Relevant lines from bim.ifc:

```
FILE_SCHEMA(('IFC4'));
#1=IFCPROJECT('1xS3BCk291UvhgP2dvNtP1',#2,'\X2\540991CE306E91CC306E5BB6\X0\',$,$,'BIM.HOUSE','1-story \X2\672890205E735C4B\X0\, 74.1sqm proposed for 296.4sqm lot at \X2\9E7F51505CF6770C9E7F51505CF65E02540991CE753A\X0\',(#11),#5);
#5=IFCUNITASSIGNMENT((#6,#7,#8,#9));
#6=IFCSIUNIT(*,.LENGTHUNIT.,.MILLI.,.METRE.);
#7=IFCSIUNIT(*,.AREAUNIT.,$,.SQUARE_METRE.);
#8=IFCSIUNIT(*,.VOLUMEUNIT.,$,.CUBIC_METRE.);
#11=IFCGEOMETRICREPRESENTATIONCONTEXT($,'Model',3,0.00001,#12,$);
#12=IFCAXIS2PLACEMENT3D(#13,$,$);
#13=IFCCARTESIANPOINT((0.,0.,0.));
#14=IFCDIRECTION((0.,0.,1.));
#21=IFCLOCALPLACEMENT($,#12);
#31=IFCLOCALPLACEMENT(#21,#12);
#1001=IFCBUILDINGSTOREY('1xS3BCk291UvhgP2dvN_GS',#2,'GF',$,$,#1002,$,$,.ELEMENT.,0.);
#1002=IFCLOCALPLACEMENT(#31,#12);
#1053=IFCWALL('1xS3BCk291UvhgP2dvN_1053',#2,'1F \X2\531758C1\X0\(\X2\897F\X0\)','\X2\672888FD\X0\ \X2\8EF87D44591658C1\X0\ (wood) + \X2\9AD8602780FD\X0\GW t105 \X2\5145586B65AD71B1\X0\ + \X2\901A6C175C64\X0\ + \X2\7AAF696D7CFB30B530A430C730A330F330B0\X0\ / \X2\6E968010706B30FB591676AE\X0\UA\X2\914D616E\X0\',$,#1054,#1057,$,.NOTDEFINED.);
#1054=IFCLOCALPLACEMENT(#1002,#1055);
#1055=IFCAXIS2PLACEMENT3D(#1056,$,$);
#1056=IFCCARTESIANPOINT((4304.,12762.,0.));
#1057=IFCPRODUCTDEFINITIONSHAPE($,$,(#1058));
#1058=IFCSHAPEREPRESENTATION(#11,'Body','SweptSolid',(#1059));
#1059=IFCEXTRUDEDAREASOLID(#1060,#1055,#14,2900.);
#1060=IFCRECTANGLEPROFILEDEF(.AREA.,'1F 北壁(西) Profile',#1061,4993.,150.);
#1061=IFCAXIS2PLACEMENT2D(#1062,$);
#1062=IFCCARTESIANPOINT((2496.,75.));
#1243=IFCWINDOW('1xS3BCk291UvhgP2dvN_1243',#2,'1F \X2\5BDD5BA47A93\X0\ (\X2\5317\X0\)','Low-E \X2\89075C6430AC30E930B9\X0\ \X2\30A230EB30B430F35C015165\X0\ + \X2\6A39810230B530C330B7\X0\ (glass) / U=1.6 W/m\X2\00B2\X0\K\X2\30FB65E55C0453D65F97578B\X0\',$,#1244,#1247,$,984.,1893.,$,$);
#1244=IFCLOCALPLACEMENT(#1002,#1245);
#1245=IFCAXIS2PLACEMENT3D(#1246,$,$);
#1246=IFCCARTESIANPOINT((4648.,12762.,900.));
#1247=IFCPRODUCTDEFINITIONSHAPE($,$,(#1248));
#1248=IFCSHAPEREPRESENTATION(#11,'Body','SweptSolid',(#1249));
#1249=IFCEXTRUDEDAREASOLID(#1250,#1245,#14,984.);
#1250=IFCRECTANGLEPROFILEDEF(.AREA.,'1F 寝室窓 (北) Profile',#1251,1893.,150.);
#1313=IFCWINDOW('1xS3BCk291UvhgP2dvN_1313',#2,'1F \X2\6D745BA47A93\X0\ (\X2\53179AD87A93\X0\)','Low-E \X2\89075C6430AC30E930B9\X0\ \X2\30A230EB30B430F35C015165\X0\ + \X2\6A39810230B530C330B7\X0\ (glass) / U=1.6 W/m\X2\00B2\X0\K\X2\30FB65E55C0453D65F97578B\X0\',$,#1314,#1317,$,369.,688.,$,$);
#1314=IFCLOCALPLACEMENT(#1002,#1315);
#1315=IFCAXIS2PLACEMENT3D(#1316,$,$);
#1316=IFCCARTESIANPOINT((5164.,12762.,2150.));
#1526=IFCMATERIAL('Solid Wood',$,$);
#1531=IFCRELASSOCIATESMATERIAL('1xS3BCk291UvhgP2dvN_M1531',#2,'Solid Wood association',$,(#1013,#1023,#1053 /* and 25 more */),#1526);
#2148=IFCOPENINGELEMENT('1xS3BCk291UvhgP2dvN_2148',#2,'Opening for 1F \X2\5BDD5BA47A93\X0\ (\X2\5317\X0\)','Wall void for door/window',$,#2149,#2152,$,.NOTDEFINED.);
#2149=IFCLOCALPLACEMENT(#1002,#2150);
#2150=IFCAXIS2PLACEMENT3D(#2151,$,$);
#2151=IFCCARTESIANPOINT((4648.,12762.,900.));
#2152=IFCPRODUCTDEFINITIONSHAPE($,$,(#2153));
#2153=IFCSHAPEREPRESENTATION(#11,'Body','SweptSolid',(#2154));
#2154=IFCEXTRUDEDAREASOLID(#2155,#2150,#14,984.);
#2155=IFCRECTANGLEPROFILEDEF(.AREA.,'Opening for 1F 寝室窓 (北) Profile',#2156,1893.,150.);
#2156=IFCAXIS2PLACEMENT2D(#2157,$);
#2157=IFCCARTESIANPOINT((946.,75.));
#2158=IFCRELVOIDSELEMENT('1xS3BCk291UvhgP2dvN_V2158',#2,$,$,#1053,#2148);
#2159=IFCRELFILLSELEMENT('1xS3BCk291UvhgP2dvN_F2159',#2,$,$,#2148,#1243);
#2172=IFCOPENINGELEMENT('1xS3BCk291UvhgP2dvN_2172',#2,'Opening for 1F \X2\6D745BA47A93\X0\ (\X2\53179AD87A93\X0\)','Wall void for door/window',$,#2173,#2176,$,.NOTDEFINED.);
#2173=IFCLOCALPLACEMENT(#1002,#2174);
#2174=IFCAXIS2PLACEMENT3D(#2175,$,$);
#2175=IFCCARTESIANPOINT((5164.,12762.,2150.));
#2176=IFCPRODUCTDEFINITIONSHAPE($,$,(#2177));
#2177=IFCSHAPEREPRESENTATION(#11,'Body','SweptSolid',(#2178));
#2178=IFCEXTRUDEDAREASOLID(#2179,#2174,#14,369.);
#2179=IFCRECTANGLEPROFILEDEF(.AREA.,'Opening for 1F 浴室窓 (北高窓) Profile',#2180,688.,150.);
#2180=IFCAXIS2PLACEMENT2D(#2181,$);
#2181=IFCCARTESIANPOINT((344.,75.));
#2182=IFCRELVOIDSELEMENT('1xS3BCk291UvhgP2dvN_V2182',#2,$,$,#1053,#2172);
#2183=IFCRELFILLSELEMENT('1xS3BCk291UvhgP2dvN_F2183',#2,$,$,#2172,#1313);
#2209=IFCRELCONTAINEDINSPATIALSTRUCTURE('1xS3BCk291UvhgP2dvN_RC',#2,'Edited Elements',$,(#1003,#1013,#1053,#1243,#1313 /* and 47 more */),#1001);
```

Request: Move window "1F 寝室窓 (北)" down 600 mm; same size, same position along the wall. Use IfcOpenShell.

```python
import numpy as np
import ifcopenshell
import ifcopenshell.api.geometry
import ifcopenshell.util.placement
import ifcopenshell.util.unit

model = ifcopenshell.open("bim.ifc")
unit_scale = ifcopenshell.util.unit.calculate_unit_scale(model)

window = model.by_guid("1xS3BCk291UvhgP2dvN_1243")
opening = window.FillsVoids[0].RelatingOpeningElement
dz = -0.6 / unit_scale

shift = np.array([0.0, 0.0, dz])
# The window is not placed relative to its opening, so move both.
for product in (opening, window):
    matrix = ifcopenshell.util.placement.get_local_placement(product.ObjectPlacement)
    matrix[:3, 3] += shift
    ifcopenshell.api.geometry.edit_object_placement(model, product=product, matrix=matrix, is_si=False)

print(f"moved by {dz * unit_scale:+.3f} m")

model.write("bim_edited.ifc")
```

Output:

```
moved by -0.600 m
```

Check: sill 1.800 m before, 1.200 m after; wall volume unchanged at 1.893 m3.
